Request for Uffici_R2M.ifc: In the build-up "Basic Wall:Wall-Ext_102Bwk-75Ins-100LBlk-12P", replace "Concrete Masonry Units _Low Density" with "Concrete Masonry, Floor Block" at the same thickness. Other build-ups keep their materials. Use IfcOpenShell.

First a look at what the model holds.

```python
import ifcopenshell
import ifcopenshell.util.element

model = ifcopenshell.open("Uffici_R2M.ifc")
print(model.schema)
for layer_set in model.by_type("IfcMaterialLayerSet"):
    if layer_set.LayerSetName == "Basic Wall:Wall-Ext_102Bwk-75Ins-100LBlk-12P":
        for layer in layer_set.MaterialLayers:
            print(layer.id(), layer.Material and layer.Material.Name, layer.LayerThickness, sep=" | ")
        print(len(ifcopenshell.util.element.get_elements_by_material(model, layer_set)), "elements and types use it")
print(sorted(m.Name for m in model.by_type("IfcMaterial") if m.Name)[:60])
```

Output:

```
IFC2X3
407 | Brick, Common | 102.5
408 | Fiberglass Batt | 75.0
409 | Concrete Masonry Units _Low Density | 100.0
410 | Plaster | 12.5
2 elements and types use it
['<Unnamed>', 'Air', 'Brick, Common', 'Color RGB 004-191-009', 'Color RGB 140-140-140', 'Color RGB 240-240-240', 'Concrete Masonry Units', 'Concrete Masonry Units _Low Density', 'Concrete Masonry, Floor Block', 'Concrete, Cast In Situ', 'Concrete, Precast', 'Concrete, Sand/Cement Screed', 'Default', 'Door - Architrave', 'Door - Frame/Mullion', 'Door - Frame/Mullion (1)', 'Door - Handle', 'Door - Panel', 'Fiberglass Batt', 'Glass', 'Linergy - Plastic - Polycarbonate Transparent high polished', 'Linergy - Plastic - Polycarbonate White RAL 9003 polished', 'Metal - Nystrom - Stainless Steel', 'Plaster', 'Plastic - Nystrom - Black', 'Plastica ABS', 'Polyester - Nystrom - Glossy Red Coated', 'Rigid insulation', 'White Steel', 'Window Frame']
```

```python
import ifcopenshell
import ifcopenshell.api.material

model = ifcopenshell.open("Uffici_R2M.ifc")

layer_set = next(s for s in model.by_type("IfcMaterialLayerSet") if s.LayerSetName == "Basic Wall:Wall-Ext_102Bwk-75Ins-100LBlk-12P")
layer = next(l for l in layer_set.MaterialLayers if l.Material and l.Material.Name == "Concrete Masonry Units _Low Density")
material = next(m for m in model.by_type("IfcMaterial") if m.Name == "Concrete Masonry, Floor Block")

# Point this one layer at the other material; renaming the old one would change it everywhere.
ifcopenshell.api.material.edit_layer(model, layer=layer, attributes={}, material=material)

print([l.Material.Name if l.Material else None for l in layer_set.MaterialLayers])

model.write("Uffici_R2M_edited.ifc")
```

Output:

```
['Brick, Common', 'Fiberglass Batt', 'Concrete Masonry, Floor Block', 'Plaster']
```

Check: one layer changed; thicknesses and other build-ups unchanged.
